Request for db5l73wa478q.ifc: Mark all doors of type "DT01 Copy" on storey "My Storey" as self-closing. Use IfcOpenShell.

First a look at what the model holds.

```python
import ifcopenshell
import ifcopenshell.util.element

model = ifcopenshell.open("db5l73wa478q.ifc")
print(model.schema)
storey = next(s for s in model.by_type("IfcBuildingStorey") if s.Name == "My Storey")
doors = [e for e in ifcopenshell.util.element.get_decomposition(storey) if e.is_a("IfcDoor")]
seen = {}
for e in doors:
    element_type = ifcopenshell.util.element.get_type(e)
    key = (element_type.Name if element_type != e and element_type else None, ifcopenshell.util.element.get_pset(e, "Pset_DoorCommon", "SelfClosing"))
    seen[key] = seen.get(key, 0) + 1
for (name, value), count in sorted(seen.items(), key=str):
    print(count, "x", name, "|", value)
```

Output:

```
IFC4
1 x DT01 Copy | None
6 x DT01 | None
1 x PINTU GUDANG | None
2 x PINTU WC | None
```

```python
import ifcopenshell
import ifcopenshell.api.pset
import ifcopenshell.util.element

model = ifcopenshell.open("db5l73wa478q.ifc")

storey = next(s for s in model.by_type("IfcBuildingStorey") if s.Name == "My Storey")
doors = [e for e in ifcopenshell.util.element.get_decomposition(storey) if e.is_a("IfcDoor")]

count = 0
for e in doors:
    element_type = ifcopenshell.util.element.get_type(e)
    if element_type in (None, e) or element_type.Name != "DT01 Copy":
        continue
    # add_pset returns the element's existing set when there is one.
    pset = ifcopenshell.api.pset.add_pset(model, product=e, name="Pset_DoorCommon")
    ifcopenshell.api.pset.edit_pset(model, pset=pset, properties={"SelfClosing": True})
    count += 1

print(count, "doors updated")

model.write("db5l73wa478q_rev.ifc")
```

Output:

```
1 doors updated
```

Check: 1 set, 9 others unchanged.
